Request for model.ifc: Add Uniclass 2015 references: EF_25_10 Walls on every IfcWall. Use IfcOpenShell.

First a look at what the model holds.

```python
import ifcopenshell

model = ifcopenshell.open("model.ifc")
print(model.schema)
print("classifications:", [c.Name for c in model.by_type("IfcClassification")])
for ifc_class in ("IfcDoor", "IfcRoof", "IfcStair", "IfcWall", "IfcWindow"):
    print(ifc_class, len(model.by_type(ifc_class)))
```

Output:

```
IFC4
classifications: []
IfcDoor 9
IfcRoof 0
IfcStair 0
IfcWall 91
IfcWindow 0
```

```python
import ifcopenshell
import ifcopenshell.api.classification

model = ifcopenshell.open("model.ifc")

system = ifcopenshell.api.classification.add_classification(model, classification="Uniclass 2015")

codes = {
    "IfcWall": ("EF_25_10", "Walls"),
}
for ifc_class, (code, name) in codes.items():
    products = model.by_type(ifc_class)
    ifcopenshell.api.classification.add_reference(
        model, products=products, classification=system, identification=code, name=name
    )
    print(code, len(products))

model.write("model-out.ifc")
```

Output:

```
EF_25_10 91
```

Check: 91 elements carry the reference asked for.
